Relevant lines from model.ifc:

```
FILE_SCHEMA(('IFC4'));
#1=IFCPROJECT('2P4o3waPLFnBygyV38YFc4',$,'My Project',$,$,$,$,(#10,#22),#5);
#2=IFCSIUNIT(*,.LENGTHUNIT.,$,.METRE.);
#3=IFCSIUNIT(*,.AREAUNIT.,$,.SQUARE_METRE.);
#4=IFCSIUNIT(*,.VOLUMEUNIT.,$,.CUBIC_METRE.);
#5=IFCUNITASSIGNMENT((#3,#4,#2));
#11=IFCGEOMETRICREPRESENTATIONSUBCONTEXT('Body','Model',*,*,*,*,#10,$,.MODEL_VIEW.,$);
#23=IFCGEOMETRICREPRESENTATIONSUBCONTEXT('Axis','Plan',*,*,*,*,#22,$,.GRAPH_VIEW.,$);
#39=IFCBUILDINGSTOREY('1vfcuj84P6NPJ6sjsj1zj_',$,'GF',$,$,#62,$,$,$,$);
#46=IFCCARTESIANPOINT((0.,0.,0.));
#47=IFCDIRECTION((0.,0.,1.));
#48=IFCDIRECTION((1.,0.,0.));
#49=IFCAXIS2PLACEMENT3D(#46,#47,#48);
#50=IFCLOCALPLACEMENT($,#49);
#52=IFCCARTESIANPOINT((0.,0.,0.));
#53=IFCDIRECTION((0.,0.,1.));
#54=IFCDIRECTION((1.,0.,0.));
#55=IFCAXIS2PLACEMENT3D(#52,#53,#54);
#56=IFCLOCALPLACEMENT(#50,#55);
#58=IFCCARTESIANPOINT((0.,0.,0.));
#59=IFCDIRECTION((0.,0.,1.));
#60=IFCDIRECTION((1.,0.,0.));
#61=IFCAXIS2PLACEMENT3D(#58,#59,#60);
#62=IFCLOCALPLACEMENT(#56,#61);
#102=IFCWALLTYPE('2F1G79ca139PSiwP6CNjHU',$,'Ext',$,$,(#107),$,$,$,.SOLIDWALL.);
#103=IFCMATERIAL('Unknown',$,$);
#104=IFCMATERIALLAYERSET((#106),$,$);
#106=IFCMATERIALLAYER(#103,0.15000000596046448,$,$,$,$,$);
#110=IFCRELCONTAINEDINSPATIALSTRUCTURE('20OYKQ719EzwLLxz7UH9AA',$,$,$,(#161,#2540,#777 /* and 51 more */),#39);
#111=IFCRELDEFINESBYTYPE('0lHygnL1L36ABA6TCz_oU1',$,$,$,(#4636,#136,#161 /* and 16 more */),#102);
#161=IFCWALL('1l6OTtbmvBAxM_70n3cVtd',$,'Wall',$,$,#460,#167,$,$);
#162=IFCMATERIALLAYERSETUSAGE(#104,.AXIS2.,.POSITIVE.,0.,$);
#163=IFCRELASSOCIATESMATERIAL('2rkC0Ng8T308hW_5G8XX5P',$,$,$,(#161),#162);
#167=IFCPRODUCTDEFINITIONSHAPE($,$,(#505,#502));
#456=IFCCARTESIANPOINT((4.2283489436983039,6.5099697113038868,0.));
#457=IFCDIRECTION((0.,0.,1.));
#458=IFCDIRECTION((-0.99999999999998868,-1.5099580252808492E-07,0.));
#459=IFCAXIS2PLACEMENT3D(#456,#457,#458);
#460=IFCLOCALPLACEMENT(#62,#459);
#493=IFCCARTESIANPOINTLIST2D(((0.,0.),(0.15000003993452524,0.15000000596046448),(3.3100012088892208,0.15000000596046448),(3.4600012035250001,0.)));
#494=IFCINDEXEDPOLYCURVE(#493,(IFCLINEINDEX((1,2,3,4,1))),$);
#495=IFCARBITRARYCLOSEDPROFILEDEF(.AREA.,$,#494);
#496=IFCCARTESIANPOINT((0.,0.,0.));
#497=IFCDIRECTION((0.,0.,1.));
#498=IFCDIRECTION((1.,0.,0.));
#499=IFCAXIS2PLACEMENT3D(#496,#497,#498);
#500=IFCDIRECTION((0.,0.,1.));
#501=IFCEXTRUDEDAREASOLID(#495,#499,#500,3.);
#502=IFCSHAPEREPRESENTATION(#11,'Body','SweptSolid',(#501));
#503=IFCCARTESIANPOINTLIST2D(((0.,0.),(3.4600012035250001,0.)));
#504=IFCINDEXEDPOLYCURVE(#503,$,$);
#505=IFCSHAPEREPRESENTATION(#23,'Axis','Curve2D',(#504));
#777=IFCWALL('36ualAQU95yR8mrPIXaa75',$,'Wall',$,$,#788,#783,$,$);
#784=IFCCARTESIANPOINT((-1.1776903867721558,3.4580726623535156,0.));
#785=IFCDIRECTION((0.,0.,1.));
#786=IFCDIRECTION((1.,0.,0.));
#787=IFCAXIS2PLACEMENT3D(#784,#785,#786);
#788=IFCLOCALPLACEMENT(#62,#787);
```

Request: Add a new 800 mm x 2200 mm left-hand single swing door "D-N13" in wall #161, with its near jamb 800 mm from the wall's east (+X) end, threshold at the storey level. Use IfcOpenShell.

```python
import numpy as np
import ifcopenshell
import ifcopenshell.api.feature
import ifcopenshell.api.geometry
import ifcopenshell.api.root
import ifcopenshell.api.spatial
import ifcopenshell.geom
import ifcopenshell.util.element
import ifcopenshell.util.placement
import ifcopenshell.util.representation
import ifcopenshell.util.shape
import ifcopenshell.util.unit

model = ifcopenshell.open("model.ifc")
unit_scale = ifcopenshell.util.unit.calculate_unit_scale(model)
settings = ifcopenshell.geom.settings()


def volume(element):
    """Net volume in cubic metres, openings subtracted."""
    shape = ifcopenshell.geom.create_shape(settings, element)
    return ifcopenshell.util.shape.get_volume(shape.geometry)


wall = model.by_id(161)
storey = ifcopenshell.util.element.get_container(wall, ifc_class="IfcBuildingStorey")
context = ifcopenshell.util.representation.get_context(model, "Model", "Body", "MODEL_VIEW")
before = volume(wall)

width, height, from_end, sill = 0.8, 2.2, 0.8, 0.0  # metres

# The wall runs along its own X axis, and the end named is its -X end.
wall_shape = ifcopenshell.geom.create_shape(settings, wall)
x, y, z = ifcopenshell.util.shape.get_vertices(wall_shape.geometry).T
start = x.min() + from_end
face, thickness = float(y.min()), float(y.max() - y.min())
wall_matrix = ifcopenshell.util.placement.get_local_placement(wall.ObjectPlacement)
level = ifcopenshell.util.placement.get_local_placement(storey.ObjectPlacement)[2, 3]


def in_wall(x, y):
    """Placement at x, y metres in the wall's axes, at sill height."""
    matrix = wall_matrix.copy()
    matrix[:, 3] = wall_matrix @ np.array([x / unit_scale, y / unit_scale, 0.0, 1.0])
    matrix[2, 3] = level + sill / unit_scale
    return matrix


# Opening: a box that overshoots both wall faces by 50 mm.
opening = ifcopenshell.api.root.create_entity(model, ifc_class="IfcOpeningElement", predefined_type="OPENING")
box = ifcopenshell.api.geometry.add_wall_representation(
    model, context=context, length=width, height=height, thickness=thickness + 0.1
)
ifcopenshell.api.geometry.assign_representation(model, product=opening, representation=box)
ifcopenshell.api.geometry.edit_object_placement(model, product=opening, matrix=in_wall(start, face - 0.05), is_si=False)
ifcopenshell.api.feature.add_feature(model, feature=opening, element=wall)

door = ifcopenshell.api.root.create_entity(model, ifc_class="IfcDoor", name="D-N13", predefined_type="DOOR")
door.OverallWidth, door.OverallHeight = width / unit_scale, height / unit_scale
door.OperationType = "SINGLE_SWING_LEFT"
body = ifcopenshell.api.geometry.add_door_representation(
    model,
    context=context,
    overall_width=door.OverallWidth,
    overall_height=door.OverallHeight,
    operation_type="SINGLE_SWING_LEFT",
    lining_properties={"LiningDepth": thickness / unit_scale, "ThresholdDepth": thickness / unit_scale},
)
ifcopenshell.api.geometry.assign_representation(model, product=door, representation=body)
ifcopenshell.api.spatial.assign_container(model, products=[door], relating_structure=storey)
ifcopenshell.api.feature.add_filling(model, opening=opening, element=door)

# The lining spans the wall, so the door starts at the wall face.
ifcopenshell.api.geometry.edit_object_placement(model, product=door, matrix=in_wall(start, face), is_si=False)

after = volume(wall)

print(f"wall volume {before:.3f} -> {after:.3f} m3")

model.write("model_rev.ifc")
```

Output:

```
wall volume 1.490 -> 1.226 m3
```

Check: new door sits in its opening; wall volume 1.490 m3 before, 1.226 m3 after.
